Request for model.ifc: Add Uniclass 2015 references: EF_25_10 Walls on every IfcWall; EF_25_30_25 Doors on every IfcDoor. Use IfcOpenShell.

First a look at what the model holds.

```python
import ifcopenshell

model = ifcopenshell.open("model.ifc")
print(model.schema)
print("classifications:", [c.Name for c in model.by_type("IfcClassification")])
for ifc_class in ("IfcDoor", "IfcRoof", "IfcStair", "IfcWall", "IfcWindow"):
    print(ifc_class, len(model.by_type(ifc_class)))
```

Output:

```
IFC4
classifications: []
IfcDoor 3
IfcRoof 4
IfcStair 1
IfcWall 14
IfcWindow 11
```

```python
import ifcopenshell
import ifcopenshell.api.classification

model = ifcopenshell.open("model.ifc")

system = ifcopenshell.api.classification.add_classification(model, classification="Uniclass 2015")

codes = {
    "IfcWall": ("EF_25_10", "Walls"),
    "IfcDoor": ("EF_25_30_25", "Doors"),
}
for ifc_class, (code, name) in codes.items():
    products = model.by_type(ifc_class)
    ifcopenshell.api.classification.add_reference(
        model, products=products, classification=system, identification=code, name=name
    )
    print(code, len(products))

model.write("model-out.ifc")
```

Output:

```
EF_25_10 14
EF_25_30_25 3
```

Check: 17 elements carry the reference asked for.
